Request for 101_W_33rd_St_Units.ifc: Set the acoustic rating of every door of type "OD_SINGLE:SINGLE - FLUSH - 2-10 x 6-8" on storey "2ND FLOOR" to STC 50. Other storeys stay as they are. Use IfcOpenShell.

First a look at what the model holds.

```python
import ifcopenshell
import ifcopenshell.util.element

model = ifcopenshell.open("101_W_33rd_St_Units.ifc")
print(model.schema)
storey = next(s for s in model.by_type("IfcBuildingStorey") if s.Name == "2ND FLOOR")
doors = [e for e in ifcopenshell.util.element.get_decomposition(storey) if e.is_a("IfcDoor")]
seen = {}
for e in doors:
    element_type = ifcopenshell.util.element.get_type(e)
    key = (element_type.Name if element_type != e and element_type else None, ifcopenshell.util.element.get_pset(e, "Pset_DoorCommon", "AcousticRating"))
    seen[key] = seen.get(key, 0) + 1
for (name, value), count in sorted(seen.items(), key=str):
    print(count, "x", name, "|", value)
```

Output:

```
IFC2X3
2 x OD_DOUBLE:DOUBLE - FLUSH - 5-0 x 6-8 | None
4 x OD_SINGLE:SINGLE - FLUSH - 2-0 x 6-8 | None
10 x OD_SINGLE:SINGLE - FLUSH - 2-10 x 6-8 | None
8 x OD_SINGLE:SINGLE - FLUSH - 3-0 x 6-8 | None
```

```python
import ifcopenshell
import ifcopenshell.api.pset
import ifcopenshell.util.element

model = ifcopenshell.open("101_W_33rd_St_Units.ifc")

storey = next(s for s in model.by_type("IfcBuildingStorey") if s.Name == "2ND FLOOR")
doors = [e for e in ifcopenshell.util.element.get_decomposition(storey) if e.is_a("IfcDoor")]

count = 0
for e in doors:
    element_type = ifcopenshell.util.element.get_type(e)
    if element_type in (None, e) or element_type.Name != "OD_SINGLE:SINGLE - FLUSH - 2-10 x 6-8":
        continue
    # add_pset returns the element's existing set when there is one.
    pset = ifcopenshell.api.pset.add_pset(model, product=e, name="Pset_DoorCommon")
    ifcopenshell.api.pset.edit_pset(model, pset=pset, properties={"AcousticRating": "STC 50"})
    count += 1

print(count, "doors updated")

model.write("101_W_33rd_St_Units-out.ifc")
```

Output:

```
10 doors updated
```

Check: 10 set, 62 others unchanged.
